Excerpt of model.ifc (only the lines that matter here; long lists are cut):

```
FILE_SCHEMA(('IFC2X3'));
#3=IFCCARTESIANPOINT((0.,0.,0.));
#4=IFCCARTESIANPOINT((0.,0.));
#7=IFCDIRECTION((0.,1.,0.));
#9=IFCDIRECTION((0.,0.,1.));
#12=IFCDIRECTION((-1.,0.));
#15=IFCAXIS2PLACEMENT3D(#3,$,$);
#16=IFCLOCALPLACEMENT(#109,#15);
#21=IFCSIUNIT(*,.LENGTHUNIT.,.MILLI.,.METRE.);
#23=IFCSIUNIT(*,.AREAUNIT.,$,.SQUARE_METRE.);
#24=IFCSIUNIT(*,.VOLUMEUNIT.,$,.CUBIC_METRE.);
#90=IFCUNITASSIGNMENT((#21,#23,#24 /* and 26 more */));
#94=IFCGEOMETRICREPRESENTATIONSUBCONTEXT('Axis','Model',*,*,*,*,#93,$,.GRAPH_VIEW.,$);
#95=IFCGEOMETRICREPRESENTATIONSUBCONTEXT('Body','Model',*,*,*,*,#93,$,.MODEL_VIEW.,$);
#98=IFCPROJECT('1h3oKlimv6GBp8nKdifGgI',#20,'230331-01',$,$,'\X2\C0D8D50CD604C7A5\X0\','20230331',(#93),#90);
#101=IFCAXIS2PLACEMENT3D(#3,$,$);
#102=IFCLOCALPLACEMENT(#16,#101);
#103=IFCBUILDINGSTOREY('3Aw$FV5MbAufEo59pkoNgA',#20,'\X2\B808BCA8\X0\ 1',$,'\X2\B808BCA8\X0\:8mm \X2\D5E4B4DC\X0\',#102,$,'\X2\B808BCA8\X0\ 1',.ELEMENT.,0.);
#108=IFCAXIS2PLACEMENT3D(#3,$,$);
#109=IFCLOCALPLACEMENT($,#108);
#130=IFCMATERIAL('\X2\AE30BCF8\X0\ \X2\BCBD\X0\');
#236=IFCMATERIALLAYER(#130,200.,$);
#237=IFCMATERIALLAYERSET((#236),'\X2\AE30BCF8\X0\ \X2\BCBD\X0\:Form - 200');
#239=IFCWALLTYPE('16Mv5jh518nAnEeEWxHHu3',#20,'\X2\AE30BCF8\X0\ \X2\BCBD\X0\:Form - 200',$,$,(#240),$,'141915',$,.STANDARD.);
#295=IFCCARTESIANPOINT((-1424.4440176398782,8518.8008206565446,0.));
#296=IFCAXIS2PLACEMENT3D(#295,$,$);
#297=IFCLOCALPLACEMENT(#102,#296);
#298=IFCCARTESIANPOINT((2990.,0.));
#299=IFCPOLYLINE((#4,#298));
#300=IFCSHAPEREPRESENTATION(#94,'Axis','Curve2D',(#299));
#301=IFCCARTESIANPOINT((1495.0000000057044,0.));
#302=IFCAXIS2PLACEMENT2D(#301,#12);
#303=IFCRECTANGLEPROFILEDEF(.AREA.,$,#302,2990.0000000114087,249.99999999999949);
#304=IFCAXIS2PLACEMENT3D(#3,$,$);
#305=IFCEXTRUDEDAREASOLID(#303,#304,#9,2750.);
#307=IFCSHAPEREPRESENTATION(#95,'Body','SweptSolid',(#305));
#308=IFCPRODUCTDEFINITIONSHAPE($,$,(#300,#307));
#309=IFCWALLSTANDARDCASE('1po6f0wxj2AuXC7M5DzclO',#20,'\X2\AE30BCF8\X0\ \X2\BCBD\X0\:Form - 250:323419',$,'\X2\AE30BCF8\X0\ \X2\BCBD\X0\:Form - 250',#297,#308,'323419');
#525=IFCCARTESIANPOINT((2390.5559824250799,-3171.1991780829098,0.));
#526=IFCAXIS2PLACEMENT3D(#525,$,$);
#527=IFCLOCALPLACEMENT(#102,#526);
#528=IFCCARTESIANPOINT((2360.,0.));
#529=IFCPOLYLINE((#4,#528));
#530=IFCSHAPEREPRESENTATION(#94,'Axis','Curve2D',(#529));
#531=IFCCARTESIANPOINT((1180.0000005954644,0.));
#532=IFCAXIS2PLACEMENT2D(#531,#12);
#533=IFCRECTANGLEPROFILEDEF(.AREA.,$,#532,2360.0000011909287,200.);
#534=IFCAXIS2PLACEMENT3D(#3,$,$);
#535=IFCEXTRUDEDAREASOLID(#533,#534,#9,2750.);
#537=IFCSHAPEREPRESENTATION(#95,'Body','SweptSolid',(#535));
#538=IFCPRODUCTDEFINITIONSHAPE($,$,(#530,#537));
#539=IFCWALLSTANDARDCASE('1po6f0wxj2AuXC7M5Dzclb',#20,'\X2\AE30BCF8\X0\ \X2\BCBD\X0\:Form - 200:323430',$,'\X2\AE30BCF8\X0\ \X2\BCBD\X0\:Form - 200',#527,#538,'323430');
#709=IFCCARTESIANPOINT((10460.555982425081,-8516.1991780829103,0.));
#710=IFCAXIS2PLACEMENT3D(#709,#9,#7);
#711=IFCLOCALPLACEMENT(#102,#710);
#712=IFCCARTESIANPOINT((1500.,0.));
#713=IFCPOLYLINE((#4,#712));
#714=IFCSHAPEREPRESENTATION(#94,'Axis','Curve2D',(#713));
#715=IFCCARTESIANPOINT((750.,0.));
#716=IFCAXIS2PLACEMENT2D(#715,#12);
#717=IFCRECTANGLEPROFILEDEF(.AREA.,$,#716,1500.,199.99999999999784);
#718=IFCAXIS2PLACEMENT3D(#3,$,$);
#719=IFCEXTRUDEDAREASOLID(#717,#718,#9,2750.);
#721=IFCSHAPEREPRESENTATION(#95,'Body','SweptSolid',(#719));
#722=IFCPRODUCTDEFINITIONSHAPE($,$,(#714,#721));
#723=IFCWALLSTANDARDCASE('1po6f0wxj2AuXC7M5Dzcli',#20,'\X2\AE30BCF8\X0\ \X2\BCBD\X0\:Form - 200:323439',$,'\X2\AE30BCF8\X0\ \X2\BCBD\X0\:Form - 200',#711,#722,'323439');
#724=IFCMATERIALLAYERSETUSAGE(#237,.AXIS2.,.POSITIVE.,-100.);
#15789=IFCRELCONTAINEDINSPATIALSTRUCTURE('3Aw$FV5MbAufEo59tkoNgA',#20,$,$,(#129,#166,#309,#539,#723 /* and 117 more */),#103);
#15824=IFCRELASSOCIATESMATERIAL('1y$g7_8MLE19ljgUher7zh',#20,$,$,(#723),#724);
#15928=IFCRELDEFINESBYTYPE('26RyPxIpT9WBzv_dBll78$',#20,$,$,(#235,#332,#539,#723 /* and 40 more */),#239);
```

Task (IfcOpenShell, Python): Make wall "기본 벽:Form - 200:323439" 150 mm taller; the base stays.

```python
import ifcopenshell
import ifcopenshell.geom
import ifcopenshell.util.representation
import ifcopenshell.util.shape
import ifcopenshell.util.unit

model = ifcopenshell.open("model.ifc")
unit_scale = ifcopenshell.util.unit.calculate_unit_scale(model)
settings = ifcopenshell.geom.settings()


def volume(element):
    """Net volume in cubic metres, openings subtracted."""
    shape = ifcopenshell.geom.create_shape(settings, element)
    return ifcopenshell.util.shape.get_volume(shape.geometry)


wall = model.by_guid("1po6f0wxj2AuXC7M5Dzcli")
before = volume(wall)

body = ifcopenshell.util.representation.get_representation(wall, "Model", "Body")
solid = body.Items[0]
old_height = solid.Depth
solid.Depth += 0.15 / unit_scale
after = volume(wall)

print(f"height {old_height:g} -> {solid.Depth:g}, volume {before:.3f} -> {after:.3f} m3")

model.write("model_updated.ifc")
```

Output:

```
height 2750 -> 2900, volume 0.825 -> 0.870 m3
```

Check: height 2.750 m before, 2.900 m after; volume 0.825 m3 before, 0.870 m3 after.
